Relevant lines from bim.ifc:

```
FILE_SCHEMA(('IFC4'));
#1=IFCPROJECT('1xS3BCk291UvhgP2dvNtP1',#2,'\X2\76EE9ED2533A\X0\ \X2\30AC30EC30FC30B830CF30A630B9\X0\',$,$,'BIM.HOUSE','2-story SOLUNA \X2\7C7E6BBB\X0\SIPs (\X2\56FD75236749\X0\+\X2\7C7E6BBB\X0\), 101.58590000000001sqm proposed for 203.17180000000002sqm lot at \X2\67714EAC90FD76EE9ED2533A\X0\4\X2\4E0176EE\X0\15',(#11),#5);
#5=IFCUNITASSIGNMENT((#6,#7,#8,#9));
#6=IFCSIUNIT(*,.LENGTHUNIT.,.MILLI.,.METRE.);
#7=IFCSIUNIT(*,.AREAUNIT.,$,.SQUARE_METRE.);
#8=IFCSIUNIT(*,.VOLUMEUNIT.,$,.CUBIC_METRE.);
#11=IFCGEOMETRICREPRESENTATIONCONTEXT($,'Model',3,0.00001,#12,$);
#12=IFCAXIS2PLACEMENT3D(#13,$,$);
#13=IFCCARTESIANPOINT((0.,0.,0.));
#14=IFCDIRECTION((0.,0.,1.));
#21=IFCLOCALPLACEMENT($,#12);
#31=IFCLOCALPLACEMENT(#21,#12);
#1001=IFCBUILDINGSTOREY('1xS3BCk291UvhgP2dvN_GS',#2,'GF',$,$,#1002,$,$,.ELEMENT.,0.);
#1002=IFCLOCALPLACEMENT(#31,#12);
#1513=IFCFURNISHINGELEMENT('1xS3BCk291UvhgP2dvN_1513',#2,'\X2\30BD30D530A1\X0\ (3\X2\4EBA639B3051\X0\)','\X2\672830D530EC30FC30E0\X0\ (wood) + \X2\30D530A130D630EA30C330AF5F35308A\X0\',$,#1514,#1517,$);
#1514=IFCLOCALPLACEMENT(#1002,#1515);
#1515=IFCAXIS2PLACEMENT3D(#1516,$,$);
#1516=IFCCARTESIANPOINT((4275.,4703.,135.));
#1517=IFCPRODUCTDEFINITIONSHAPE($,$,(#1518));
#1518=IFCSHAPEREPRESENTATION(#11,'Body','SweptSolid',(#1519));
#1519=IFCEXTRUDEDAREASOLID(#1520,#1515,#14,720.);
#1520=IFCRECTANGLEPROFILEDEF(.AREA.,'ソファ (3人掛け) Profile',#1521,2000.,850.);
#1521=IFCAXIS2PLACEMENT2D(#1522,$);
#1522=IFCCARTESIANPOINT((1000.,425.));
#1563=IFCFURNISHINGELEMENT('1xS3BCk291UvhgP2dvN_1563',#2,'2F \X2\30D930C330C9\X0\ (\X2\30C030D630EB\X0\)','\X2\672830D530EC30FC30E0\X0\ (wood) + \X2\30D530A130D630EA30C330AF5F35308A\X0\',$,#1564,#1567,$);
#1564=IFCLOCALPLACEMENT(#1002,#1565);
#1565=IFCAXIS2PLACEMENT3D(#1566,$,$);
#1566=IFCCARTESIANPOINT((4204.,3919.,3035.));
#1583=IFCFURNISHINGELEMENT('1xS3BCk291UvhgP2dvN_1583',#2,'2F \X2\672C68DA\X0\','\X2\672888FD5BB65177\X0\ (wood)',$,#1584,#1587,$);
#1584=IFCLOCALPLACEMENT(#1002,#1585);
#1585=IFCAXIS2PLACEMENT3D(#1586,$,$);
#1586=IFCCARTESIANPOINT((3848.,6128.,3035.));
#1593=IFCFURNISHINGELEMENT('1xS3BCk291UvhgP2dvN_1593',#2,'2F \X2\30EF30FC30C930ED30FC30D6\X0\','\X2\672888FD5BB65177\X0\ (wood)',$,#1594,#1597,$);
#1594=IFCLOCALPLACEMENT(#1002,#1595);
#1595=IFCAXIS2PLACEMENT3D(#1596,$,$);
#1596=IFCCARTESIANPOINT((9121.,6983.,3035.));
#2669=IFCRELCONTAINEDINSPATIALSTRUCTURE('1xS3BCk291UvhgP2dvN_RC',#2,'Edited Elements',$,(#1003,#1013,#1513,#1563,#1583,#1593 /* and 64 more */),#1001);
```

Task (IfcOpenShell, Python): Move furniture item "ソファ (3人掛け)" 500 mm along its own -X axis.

```python
import ifcopenshell
import ifcopenshell.api.geometry
import ifcopenshell.util.placement

model = ifcopenshell.open("bim.ifc")

item = model.by_guid("1xS3BCk291UvhgP2dvN_1513")
matrix = ifcopenshell.util.placement.get_local_placement(item.ObjectPlacement)
matrix[:3, 3] -= matrix[:3, 0] * 500.0
ifcopenshell.api.geometry.edit_object_placement(model, product=item, matrix=matrix, is_si=False)

print(ifcopenshell.util.placement.get_local_placement(item.ObjectPlacement).round(3) + 0.0)

model.write("bim-out.ifc")
```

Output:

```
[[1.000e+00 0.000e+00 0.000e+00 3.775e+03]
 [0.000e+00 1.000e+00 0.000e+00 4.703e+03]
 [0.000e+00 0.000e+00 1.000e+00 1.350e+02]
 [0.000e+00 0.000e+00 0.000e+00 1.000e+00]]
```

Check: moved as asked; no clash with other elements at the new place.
